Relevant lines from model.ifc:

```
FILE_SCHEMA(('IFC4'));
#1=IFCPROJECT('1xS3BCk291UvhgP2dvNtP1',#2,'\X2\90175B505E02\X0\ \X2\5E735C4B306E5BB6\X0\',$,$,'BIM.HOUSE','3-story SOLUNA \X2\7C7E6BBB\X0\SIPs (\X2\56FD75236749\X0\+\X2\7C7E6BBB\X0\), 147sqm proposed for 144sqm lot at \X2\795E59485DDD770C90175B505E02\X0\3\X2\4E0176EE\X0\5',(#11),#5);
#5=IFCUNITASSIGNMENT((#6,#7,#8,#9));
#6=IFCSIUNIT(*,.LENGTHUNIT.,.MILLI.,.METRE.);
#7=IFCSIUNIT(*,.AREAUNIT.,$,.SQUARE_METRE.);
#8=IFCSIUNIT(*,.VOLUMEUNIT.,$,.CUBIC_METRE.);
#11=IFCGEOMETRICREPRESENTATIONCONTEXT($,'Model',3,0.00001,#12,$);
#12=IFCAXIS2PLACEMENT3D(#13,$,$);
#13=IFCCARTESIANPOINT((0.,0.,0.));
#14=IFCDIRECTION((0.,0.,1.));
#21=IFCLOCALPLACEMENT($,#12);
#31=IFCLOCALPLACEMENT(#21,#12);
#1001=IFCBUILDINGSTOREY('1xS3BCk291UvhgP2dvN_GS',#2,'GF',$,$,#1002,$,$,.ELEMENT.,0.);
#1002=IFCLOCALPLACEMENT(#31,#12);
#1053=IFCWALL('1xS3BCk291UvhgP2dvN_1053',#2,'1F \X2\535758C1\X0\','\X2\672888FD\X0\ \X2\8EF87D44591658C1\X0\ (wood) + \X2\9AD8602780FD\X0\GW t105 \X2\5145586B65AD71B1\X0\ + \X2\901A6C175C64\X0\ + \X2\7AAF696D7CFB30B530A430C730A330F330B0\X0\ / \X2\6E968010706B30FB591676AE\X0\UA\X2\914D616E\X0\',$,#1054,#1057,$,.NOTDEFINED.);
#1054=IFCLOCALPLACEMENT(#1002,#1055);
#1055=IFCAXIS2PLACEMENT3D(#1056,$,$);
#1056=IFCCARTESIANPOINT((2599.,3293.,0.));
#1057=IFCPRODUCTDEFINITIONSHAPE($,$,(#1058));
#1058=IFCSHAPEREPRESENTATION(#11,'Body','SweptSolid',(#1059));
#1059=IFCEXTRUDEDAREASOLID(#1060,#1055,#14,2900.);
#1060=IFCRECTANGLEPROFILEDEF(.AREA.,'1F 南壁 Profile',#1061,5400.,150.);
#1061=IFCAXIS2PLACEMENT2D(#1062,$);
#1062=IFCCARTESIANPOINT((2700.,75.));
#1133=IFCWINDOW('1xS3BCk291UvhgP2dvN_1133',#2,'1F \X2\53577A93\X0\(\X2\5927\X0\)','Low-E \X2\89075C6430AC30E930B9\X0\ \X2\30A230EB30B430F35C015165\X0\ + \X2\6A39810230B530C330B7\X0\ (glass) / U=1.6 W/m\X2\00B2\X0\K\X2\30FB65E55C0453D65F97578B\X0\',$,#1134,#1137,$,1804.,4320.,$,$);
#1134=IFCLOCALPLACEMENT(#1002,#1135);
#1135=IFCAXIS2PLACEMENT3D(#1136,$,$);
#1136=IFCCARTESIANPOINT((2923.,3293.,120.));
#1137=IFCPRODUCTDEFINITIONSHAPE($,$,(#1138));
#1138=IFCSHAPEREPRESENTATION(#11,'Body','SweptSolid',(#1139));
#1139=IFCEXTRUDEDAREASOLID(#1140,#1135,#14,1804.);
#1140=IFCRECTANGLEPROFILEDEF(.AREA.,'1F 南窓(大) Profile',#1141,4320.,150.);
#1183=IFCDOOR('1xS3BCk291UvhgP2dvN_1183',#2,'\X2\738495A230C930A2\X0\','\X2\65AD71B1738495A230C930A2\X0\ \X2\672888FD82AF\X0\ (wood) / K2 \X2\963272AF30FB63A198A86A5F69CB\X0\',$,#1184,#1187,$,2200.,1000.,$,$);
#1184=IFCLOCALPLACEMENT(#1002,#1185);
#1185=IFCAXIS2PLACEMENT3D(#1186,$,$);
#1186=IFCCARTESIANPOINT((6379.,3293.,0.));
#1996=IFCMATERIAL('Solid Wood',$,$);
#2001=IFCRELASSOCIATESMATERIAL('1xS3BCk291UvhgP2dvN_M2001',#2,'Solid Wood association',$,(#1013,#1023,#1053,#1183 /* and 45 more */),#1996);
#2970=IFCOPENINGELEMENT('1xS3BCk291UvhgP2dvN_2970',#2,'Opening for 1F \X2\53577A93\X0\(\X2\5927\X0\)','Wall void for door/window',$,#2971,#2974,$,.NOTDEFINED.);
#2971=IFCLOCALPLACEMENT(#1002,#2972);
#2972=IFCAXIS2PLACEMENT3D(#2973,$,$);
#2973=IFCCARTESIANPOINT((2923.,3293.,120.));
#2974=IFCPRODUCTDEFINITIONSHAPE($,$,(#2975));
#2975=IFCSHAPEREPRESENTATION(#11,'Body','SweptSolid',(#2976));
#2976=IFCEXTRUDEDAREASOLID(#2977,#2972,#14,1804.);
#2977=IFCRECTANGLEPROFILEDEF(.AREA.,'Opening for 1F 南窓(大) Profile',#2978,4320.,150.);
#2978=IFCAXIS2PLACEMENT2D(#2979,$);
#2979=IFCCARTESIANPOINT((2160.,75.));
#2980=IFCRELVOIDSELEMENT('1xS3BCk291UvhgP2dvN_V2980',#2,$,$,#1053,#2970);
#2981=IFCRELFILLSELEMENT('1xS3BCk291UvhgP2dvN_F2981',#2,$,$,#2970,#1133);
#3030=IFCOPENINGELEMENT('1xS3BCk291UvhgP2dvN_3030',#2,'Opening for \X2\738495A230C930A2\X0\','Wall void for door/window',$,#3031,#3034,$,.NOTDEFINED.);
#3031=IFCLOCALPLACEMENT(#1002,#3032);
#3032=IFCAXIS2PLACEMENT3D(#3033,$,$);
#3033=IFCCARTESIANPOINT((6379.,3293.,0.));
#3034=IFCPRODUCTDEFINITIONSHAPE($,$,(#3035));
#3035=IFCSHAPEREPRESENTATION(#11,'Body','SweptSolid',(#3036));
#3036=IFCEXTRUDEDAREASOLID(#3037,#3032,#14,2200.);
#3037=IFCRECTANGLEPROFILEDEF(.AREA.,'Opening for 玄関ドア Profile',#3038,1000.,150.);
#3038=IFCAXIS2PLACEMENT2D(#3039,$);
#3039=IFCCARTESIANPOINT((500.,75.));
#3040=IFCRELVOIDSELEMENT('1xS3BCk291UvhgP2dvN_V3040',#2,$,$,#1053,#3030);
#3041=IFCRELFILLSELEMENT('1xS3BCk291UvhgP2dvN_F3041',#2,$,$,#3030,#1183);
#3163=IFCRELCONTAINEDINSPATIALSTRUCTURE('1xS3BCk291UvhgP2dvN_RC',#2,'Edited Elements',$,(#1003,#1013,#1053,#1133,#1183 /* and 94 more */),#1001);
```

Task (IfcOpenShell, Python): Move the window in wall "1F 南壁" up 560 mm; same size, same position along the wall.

```python
import numpy as np
import ifcopenshell
import ifcopenshell.api.geometry
import ifcopenshell.util.placement
import ifcopenshell.util.unit

model = ifcopenshell.open("model.ifc")
unit_scale = ifcopenshell.util.unit.calculate_unit_scale(model)

window = model.by_guid("1xS3BCk291UvhgP2dvN_1133")
opening = window.FillsVoids[0].RelatingOpeningElement
dz = 560.0

shift = np.array([0.0, 0.0, dz])
# The window is not placed relative to its opening, so move both.
for product in (opening, window):
    matrix = ifcopenshell.util.placement.get_local_placement(product.ObjectPlacement)
    matrix[:3, 3] += shift
    ifcopenshell.api.geometry.edit_object_placement(model, product=product, matrix=matrix, is_si=False)

print(f"moved by {dz * unit_scale:+.3f} m")

model.write("model_edited.ifc")
```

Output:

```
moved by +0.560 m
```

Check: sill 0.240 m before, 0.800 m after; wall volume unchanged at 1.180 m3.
